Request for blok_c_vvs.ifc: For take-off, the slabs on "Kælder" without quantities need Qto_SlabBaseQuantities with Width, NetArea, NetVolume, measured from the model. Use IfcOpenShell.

First a look at what the model holds.

```python
import ifcopenshell
import ifcopenshell.util.element
import ifcopenshell.util.unit

model = ifcopenshell.open("blok_c_vvs.ifc")
print(model.schema)
for unit_type in ("LENGTHUNIT", "AREAUNIT", "VOLUMEUNIT"):
    print(unit_type, ifcopenshell.util.unit.calculate_unit_scale(model, unit_type))
storey = next(s for s in model.by_type("IfcBuildingStorey") if s.Name == "Kælder")
slabs = [e for e in ifcopenshell.util.element.get_decomposition(storey) if e.is_a("IfcSlab")]
for e in sorted(slabs, key=lambda e: e.id()):
    print(e.id(), e.is_a(), e.Name, list(ifcopenshell.util.element.get_psets(e, qtos_only=True)), sep=" | ")
```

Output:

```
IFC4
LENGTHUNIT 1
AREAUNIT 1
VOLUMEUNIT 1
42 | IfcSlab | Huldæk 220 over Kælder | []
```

```python
import ifcopenshell
import ifcopenshell.api.pset
import ifcopenshell.geom
import ifcopenshell.util.element
import ifcopenshell.util.shape
import ifcopenshell.util.unit

model = ifcopenshell.open("blok_c_vvs.ifc")
unit_scale = ifcopenshell.util.unit.calculate_unit_scale(model)
area_scale = ifcopenshell.util.unit.calculate_unit_scale(model, "AREAUNIT")
volume_scale = ifcopenshell.util.unit.calculate_unit_scale(model, "VOLUMEUNIT")
settings = ifcopenshell.geom.settings()

storey = next(s for s in model.by_type("IfcBuildingStorey") if s.Name == "Kælder")
slabs = [e for e in ifcopenshell.util.element.get_decomposition(storey) if e.is_a("IfcSlab")]

for e in sorted(slabs, key=lambda e: e.id()):
    if ifcopenshell.util.element.get_psets(e, qtos_only=True, should_inherit=False):
        continue
    # Geometry comes back in metres, in the element's own axes.
    shape = ifcopenshell.geom.create_shape(settings, e)
    values = {
        "Width": ifcopenshell.util.shape.get_z(shape.geometry) / unit_scale,
        "NetArea": ifcopenshell.util.shape.get_footprint_area(shape.geometry) / area_scale,
        "NetVolume": ifcopenshell.util.shape.get_volume(shape.geometry) / volume_scale,
    }
    qto = ifcopenshell.api.pset.add_qto(model, product=e, name="Qto_SlabBaseQuantities")
    ifcopenshell.api.pset.edit_qto(model, qto=qto, properties=values)
    print(e.id(), {k: round(v, 3) for k, v in values.items()})

model.write("blok_c_vvs_updated.ifc")
```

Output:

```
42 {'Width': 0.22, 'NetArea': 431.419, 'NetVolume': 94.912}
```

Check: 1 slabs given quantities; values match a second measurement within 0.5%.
